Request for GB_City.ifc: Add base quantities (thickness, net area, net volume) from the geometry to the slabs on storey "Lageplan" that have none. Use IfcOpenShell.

First a look at what the model holds.

```python
import ifcopenshell
import ifcopenshell.util.element
import ifcopenshell.util.unit

model = ifcopenshell.open("GB_City.ifc")
print(model.schema)
for unit_type in ("LENGTHUNIT", "AREAUNIT", "VOLUMEUNIT"):
    print(unit_type, ifcopenshell.util.unit.calculate_unit_scale(model, unit_type))
storey = next(s for s in model.by_type("IfcBuildingStorey") if s.Name == "Lageplan")
slabs = [e for e in ifcopenshell.util.element.get_decomposition(storey) if e.is_a("IfcSlab")]
for e in sorted(slabs, key=lambda e: e.id()):
    print(e.id(), e.is_a(), e.Name, list(ifcopenshell.util.element.get_psets(e, qtos_only=True)), sep=" | ")
```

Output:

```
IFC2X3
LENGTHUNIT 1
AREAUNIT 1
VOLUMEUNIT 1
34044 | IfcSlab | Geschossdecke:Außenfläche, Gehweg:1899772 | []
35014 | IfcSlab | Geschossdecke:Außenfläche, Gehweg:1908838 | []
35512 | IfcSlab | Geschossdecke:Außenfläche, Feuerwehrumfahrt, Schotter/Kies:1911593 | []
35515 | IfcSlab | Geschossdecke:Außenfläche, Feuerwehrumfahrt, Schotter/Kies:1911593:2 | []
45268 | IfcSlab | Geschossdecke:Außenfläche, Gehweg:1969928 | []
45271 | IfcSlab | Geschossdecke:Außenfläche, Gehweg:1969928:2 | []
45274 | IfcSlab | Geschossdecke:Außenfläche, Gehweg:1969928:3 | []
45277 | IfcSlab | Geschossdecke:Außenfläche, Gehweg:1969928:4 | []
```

```python
import ifcopenshell
import ifcopenshell.api.pset
import ifcopenshell.geom
import ifcopenshell.util.element
import ifcopenshell.util.shape
import ifcopenshell.util.unit

model = ifcopenshell.open("GB_City.ifc")
unit_scale = ifcopenshell.util.unit.calculate_unit_scale(model)
area_scale = ifcopenshell.util.unit.calculate_unit_scale(model, "AREAUNIT")
volume_scale = ifcopenshell.util.unit.calculate_unit_scale(model, "VOLUMEUNIT")
settings = ifcopenshell.geom.settings()

storey = next(s for s in model.by_type("IfcBuildingStorey") if s.Name == "Lageplan")
slabs = [e for e in ifcopenshell.util.element.get_decomposition(storey) if e.is_a("IfcSlab")]

for e in sorted(slabs, key=lambda e: e.id()):
    if ifcopenshell.util.element.get_psets(e, qtos_only=True, should_inherit=False):
        continue
    # Geometry comes back in metres, in the element's own axes.
    shape = ifcopenshell.geom.create_shape(settings, e)
    values = {
        "Width": ifcopenshell.util.shape.get_z(shape.geometry) / unit_scale,
        "NetArea": ifcopenshell.util.shape.get_footprint_area(shape.geometry) / area_scale,
        "NetVolume": ifcopenshell.util.shape.get_volume(shape.geometry) / volume_scale,
    }
    qto = ifcopenshell.api.pset.add_qto(model, product=e, name="BaseQuantities")
    ifcopenshell.api.pset.edit_qto(model, qto=qto, properties=values)
    print(e.id(), {k: round(v, 3) for k, v in values.items()})

model.write("GB_City_edited.ifc")
```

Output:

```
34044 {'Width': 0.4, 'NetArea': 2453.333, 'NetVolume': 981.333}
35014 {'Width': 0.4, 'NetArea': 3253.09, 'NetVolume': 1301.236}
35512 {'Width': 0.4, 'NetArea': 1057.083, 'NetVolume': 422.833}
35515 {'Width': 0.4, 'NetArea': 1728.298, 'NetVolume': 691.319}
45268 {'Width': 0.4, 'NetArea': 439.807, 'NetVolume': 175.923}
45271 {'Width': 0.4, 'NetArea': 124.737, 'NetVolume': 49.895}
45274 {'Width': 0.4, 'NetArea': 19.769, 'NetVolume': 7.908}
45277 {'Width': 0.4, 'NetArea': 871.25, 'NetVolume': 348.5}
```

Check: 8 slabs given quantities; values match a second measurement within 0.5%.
